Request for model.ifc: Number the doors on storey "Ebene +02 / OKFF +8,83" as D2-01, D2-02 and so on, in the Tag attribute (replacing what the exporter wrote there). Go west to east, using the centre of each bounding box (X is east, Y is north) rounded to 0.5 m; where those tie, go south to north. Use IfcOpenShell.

First a look at what the model holds.

```python
import ifcopenshell
import ifcopenshell.util.element
import ifcopenshell.util.placement

model = ifcopenshell.open("model.ifc")
print(model.schema)
storey = next(s for s in model.by_type("IfcBuildingStorey") if s.Name == "Ebene +02 / OKFF +8,83")
doors = [e for e in ifcopenshell.util.element.get_decomposition(storey) if e.is_a("IfcDoor")]
for e in sorted(doors, key=lambda e: e.id()):
    origin = ifcopenshell.util.placement.get_local_placement(e.ObjectPlacement)[:3, 3]
    print(e.id(), e.Tag, e.Name, origin.round(2) + 0.0, sep=" | ")
```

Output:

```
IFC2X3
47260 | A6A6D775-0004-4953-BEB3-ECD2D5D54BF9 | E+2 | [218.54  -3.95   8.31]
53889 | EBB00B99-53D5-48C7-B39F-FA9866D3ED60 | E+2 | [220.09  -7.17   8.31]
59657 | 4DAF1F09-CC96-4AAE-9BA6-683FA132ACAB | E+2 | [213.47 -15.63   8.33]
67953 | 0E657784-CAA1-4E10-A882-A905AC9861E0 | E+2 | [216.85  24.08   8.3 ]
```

```python
import ifcopenshell
import ifcopenshell.geom
import ifcopenshell.util.element
import ifcopenshell.util.shape

model = ifcopenshell.open("model.ifc")
settings = ifcopenshell.geom.settings()
settings.set("use-world-coords", True)


def centre(element):
    shape = ifcopenshell.geom.create_shape(settings, element)
    return ifcopenshell.util.shape.get_bbox_centroid(shape.geometry)


storey = next(s for s in model.by_type("IfcBuildingStorey") if s.Name == "Ebene +02 / OKFF +8,83")
doors = [e for e in ifcopenshell.util.element.get_decomposition(storey) if e.is_a("IfcDoor")]

# Insertion points can sit at a corner or the storey origin, so sort by the geometry (in metres).
centres = {e: centre(e) for e in doors}
doors.sort(key=lambda e: (round(centres[e][0] / 0.5), centres[e][1]))

for i, e in enumerate(doors, start=1):
    number = f"D2-{i:02d}"
    e.Tag = number
    print(e.id(), number)

model.write("model-out.ifc")
```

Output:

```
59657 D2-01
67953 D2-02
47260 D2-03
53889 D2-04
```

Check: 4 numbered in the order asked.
